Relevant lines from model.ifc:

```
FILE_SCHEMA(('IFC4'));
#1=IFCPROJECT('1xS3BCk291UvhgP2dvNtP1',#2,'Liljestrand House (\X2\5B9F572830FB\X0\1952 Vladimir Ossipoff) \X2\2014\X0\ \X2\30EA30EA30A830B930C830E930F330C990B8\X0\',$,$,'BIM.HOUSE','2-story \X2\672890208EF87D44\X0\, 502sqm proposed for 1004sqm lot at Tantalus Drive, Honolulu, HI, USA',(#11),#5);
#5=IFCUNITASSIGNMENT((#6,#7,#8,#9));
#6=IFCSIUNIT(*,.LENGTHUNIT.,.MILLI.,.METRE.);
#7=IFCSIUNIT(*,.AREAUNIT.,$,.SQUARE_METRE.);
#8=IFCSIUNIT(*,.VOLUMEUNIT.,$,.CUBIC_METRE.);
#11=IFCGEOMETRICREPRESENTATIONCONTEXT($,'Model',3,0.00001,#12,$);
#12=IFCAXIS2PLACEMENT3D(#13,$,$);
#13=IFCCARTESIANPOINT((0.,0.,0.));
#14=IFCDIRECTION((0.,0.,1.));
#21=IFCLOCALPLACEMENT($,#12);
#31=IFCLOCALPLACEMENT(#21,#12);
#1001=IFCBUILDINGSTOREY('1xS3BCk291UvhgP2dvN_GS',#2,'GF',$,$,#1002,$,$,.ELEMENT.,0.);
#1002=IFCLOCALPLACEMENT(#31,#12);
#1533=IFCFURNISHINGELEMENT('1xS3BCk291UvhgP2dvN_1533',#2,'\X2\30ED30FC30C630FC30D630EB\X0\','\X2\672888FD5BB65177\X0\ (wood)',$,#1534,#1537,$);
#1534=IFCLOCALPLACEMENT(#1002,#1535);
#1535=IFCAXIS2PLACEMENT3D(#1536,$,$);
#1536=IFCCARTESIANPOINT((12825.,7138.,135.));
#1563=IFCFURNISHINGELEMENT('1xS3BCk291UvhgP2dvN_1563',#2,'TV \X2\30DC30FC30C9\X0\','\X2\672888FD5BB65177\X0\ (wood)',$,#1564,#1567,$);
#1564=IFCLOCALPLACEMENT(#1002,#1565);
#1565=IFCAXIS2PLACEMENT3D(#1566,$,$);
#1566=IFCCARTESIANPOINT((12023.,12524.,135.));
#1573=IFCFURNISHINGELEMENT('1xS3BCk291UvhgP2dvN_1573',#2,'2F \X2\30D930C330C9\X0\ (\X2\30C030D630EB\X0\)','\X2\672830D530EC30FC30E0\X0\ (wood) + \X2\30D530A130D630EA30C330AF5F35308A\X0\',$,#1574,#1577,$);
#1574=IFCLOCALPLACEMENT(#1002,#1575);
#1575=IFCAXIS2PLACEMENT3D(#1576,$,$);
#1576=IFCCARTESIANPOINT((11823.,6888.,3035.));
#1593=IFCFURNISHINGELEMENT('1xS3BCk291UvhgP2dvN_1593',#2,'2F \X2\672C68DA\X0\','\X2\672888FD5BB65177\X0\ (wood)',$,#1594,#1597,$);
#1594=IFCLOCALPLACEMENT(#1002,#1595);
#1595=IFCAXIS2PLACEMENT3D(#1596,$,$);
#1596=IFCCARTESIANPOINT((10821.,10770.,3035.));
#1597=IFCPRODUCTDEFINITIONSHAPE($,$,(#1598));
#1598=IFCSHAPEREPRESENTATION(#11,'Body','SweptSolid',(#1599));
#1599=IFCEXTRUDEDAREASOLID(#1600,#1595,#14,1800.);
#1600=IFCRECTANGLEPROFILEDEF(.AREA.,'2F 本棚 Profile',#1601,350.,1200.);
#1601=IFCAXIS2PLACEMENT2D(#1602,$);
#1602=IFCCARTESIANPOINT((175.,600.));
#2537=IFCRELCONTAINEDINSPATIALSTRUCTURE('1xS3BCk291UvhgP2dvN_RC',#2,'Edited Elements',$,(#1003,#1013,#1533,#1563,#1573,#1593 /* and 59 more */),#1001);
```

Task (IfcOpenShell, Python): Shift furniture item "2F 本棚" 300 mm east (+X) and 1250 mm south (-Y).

```python
import ifcopenshell
import ifcopenshell.api.geometry
import ifcopenshell.util.placement
import ifcopenshell.util.unit

model = ifcopenshell.open("model.ifc")
unit_scale = ifcopenshell.util.unit.calculate_unit_scale(model)

item = model.by_guid("1xS3BCk291UvhgP2dvN_1593")
matrix = ifcopenshell.util.placement.get_local_placement(item.ObjectPlacement)
matrix[0, 3] += 0.3 / unit_scale
matrix[1, 3] -= 1.25 / unit_scale
ifcopenshell.api.geometry.edit_object_placement(model, product=item, matrix=matrix, is_si=False)

print(ifcopenshell.util.placement.get_local_placement(item.ObjectPlacement).round(3) + 0.0)

model.write("model_v2.ifc")
```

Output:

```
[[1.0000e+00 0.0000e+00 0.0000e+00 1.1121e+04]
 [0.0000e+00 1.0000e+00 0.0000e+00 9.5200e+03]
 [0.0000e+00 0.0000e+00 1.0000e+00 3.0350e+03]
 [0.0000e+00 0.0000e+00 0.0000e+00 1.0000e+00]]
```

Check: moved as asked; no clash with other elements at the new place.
